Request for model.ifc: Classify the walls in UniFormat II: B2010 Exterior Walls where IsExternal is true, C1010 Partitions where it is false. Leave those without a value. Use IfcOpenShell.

First a look at what the model holds.

```python
import ifcopenshell
import ifcopenshell.util.element

model = ifcopenshell.open("model.ifc")
print(model.schema)
print("classifications:", [c.Name for c in model.by_type("IfcClassification")])
values = [ifcopenshell.util.element.get_pset(e, "Pset_WallCommon", "IsExternal") for e in model.by_type("IfcWall")]
for value in (True, False, None):
    print("IsExternal", value, values.count(value))
```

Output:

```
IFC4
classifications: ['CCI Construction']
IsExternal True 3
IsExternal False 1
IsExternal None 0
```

```python
import ifcopenshell
import ifcopenshell.api.classification
import ifcopenshell.util.element

model = ifcopenshell.open("model.ifc")

system = ifcopenshell.api.classification.add_classification(model, classification="UniFormat II")

walls = model.by_type("IfcWall")
external = {e: ifcopenshell.util.element.get_pset(e, "Pset_WallCommon", "IsExternal") for e in walls}
for flag, code, name in ((True, "B2010", "Exterior Walls"), (False, "C1010", "Partitions")):
    products = [e for e in walls if external[e] is flag]
    ifcopenshell.api.classification.add_reference(
        model, products=products, classification=system, identification=code, name=name
    )
    print(code, len(products))

model.write("model_updated.ifc")
```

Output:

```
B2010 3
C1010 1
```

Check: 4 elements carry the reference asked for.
